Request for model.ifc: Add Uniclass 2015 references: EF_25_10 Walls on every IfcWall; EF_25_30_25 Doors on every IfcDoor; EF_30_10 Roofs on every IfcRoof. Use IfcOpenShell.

First a look at what the model holds.

```python
import ifcopenshell

model = ifcopenshell.open("model.ifc")
print(model.schema)
print("classifications:", [c.Name for c in model.by_type("IfcClassification")])
for ifc_class in ("IfcDoor", "IfcRoof", "IfcStair", "IfcWall", "IfcWindow"):
    print(ifc_class, len(model.by_type(ifc_class)))
```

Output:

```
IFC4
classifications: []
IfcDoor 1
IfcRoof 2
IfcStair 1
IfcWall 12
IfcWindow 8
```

```python
import ifcopenshell
import ifcopenshell.api.classification

model = ifcopenshell.open("model.ifc")

system = ifcopenshell.api.classification.add_classification(model, classification="Uniclass 2015")

codes = {
    "IfcWall": ("EF_25_10", "Walls"),
    "IfcDoor": ("EF_25_30_25", "Doors"),
    "IfcRoof": ("EF_30_10", "Roofs"),
}
for ifc_class, (code, name) in codes.items():
    products = model.by_type(ifc_class)
    ifcopenshell.api.classification.add_reference(
        model, products=products, classification=system, identification=code, name=name
    )
    print(code, len(products))

model.write("model-out.ifc")
```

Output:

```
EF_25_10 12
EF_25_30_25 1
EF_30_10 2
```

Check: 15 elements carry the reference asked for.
